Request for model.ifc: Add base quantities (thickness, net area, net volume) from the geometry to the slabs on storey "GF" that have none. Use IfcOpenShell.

First a look at what the model holds.

```python
import ifcopenshell
import ifcopenshell.util.element
import ifcopenshell.util.unit

model = ifcopenshell.open("model.ifc")
print(model.schema)
for unit_type in ("LENGTHUNIT", "AREAUNIT", "VOLUMEUNIT"):
    print(unit_type, ifcopenshell.util.unit.calculate_unit_scale(model, unit_type))
storey = next(s for s in model.by_type("IfcBuildingStorey") if s.Name == "GF")
slabs = [e for e in ifcopenshell.util.element.get_decomposition(storey) if e.is_a("IfcSlab")]
for e in sorted(slabs, key=lambda e: e.id()):
    print(e.id(), e.is_a(), e.Name, list(ifcopenshell.util.element.get_psets(e, qtos_only=True)), sep=" | ")
```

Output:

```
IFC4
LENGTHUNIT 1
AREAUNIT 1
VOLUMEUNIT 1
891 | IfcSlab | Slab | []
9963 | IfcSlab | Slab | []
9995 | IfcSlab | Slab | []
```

```python
import ifcopenshell
import ifcopenshell.api.pset
import ifcopenshell.geom
import ifcopenshell.util.element
import ifcopenshell.util.shape
import ifcopenshell.util.unit

model = ifcopenshell.open("model.ifc")
unit_scale = ifcopenshell.util.unit.calculate_unit_scale(model)
area_scale = ifcopenshell.util.unit.calculate_unit_scale(model, "AREAUNIT")
volume_scale = ifcopenshell.util.unit.calculate_unit_scale(model, "VOLUMEUNIT")
settings = ifcopenshell.geom.settings()

storey = next(s for s in model.by_type("IfcBuildingStorey") if s.Name == "GF")
slabs = [e for e in ifcopenshell.util.element.get_decomposition(storey) if e.is_a("IfcSlab")]

for e in sorted(slabs, key=lambda e: e.id()):
    if ifcopenshell.util.element.get_psets(e, qtos_only=True, should_inherit=False):
        continue
    # Geometry comes back in metres, in the element's own axes.
    shape = ifcopenshell.geom.create_shape(settings, e)
    values = {
        "Width": ifcopenshell.util.shape.get_z(shape.geometry) / unit_scale,
        "NetArea": ifcopenshell.util.shape.get_footprint_area(shape.geometry) / area_scale,
        "NetVolume": ifcopenshell.util.shape.get_volume(shape.geometry) / volume_scale,
    }
    qto = ifcopenshell.api.pset.add_qto(model, product=e, name="Qto_SlabBaseQuantities")
    ifcopenshell.api.pset.edit_qto(model, qto=qto, properties=values)
    print(e.id(), {k: round(v, 3) for k, v in values.items()})

model.write("model_v2.ifc")
```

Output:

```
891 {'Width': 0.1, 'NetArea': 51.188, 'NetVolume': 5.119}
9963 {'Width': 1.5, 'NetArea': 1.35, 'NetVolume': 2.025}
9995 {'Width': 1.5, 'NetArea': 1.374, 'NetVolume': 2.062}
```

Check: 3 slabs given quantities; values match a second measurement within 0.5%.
